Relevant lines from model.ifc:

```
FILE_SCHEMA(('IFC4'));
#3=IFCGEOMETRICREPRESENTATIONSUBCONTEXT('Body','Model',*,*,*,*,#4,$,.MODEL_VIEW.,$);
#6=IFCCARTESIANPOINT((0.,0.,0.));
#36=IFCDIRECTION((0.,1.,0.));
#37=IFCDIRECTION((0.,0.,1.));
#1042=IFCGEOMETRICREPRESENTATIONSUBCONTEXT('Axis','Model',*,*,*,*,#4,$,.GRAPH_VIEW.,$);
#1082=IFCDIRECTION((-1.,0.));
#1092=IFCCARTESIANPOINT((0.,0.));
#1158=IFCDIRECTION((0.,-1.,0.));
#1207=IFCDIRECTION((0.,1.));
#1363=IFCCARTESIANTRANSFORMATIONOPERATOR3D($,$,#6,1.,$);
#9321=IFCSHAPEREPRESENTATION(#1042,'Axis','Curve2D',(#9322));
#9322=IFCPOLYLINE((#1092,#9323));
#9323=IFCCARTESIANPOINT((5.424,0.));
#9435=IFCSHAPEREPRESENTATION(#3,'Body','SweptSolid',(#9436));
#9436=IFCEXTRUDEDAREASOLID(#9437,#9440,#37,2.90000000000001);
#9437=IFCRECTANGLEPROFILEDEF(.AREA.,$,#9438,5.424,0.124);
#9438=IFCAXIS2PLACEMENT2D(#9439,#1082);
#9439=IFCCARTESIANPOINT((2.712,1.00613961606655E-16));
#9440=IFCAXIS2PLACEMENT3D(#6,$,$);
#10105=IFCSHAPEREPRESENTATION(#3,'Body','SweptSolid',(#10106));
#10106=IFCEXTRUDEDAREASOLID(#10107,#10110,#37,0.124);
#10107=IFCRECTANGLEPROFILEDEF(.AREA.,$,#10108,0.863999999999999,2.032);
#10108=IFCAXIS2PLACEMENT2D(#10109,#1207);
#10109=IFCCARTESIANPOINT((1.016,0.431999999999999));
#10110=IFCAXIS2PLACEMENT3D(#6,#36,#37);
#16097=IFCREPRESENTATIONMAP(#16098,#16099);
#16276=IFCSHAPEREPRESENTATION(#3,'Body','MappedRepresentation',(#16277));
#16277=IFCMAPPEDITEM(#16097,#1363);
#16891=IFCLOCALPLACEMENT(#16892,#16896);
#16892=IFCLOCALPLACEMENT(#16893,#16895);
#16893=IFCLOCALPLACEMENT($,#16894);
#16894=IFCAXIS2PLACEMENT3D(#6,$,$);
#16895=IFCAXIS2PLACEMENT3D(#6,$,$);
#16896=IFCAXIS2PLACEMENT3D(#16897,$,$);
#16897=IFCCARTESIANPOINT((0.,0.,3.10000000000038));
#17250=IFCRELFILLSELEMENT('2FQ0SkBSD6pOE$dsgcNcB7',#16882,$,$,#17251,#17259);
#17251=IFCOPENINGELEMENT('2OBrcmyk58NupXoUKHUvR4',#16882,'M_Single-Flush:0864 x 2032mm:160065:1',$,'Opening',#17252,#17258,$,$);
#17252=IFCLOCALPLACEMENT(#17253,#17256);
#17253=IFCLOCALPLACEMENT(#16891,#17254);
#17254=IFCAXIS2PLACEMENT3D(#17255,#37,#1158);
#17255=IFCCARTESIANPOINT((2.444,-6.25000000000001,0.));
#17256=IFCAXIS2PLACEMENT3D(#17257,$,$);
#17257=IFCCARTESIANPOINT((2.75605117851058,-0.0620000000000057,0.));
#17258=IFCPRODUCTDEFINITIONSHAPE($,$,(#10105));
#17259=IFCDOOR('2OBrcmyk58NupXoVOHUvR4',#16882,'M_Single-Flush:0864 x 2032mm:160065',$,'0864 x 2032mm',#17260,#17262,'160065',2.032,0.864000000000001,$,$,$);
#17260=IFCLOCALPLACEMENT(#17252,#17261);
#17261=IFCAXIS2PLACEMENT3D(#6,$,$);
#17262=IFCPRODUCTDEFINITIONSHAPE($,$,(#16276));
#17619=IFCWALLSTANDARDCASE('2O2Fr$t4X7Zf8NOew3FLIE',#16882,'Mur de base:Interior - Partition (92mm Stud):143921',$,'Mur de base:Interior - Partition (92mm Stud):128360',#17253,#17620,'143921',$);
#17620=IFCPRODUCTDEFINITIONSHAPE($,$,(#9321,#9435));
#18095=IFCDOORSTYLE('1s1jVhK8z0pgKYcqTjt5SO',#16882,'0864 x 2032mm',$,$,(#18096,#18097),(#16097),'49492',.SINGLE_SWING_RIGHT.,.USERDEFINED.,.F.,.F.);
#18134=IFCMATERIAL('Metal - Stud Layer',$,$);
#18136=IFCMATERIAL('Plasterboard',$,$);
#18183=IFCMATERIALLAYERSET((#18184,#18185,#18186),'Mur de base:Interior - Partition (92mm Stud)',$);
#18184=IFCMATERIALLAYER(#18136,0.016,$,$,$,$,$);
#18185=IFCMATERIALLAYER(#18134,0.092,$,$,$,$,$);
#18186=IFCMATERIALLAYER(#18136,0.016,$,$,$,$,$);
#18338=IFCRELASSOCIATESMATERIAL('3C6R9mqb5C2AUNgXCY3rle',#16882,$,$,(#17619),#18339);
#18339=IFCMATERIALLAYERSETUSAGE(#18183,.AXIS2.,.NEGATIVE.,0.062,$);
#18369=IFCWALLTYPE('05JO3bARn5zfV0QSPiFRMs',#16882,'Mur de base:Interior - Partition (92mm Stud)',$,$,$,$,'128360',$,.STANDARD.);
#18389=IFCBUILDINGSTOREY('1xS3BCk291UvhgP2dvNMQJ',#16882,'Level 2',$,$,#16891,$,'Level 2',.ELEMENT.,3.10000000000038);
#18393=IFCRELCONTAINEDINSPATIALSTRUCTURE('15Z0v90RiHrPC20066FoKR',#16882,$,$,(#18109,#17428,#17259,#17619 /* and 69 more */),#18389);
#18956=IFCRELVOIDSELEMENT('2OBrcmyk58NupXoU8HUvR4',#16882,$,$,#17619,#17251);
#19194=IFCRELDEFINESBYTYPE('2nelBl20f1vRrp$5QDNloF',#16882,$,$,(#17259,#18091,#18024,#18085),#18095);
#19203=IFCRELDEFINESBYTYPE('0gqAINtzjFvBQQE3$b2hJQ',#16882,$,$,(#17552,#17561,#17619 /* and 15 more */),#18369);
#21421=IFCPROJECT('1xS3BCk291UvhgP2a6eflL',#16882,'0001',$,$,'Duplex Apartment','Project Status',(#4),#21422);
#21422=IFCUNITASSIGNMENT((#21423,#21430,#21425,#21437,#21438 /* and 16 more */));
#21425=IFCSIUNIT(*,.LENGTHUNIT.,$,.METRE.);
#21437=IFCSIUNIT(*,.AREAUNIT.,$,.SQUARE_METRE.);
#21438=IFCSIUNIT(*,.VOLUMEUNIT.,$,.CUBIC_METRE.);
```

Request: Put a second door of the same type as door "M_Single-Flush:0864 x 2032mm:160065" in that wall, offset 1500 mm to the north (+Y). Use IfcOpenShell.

```python
import ifcopenshell
import ifcopenshell.api.feature
import ifcopenshell.api.geometry
import ifcopenshell.api.root
import ifcopenshell.geom
import ifcopenshell.util.element
import ifcopenshell.util.placement
import ifcopenshell.util.shape

model = ifcopenshell.open("model.ifc")
settings = ifcopenshell.geom.settings()


def volume(element):
    """Net volume in cubic metres, openings subtracted."""
    shape = ifcopenshell.geom.create_shape(settings, element)
    return ifcopenshell.util.shape.get_volume(shape.geometry)


def reuse_history(source, copy):
    """copy_class also copies each property set's owner history, people and application; keep the originals."""
    for rel in copy.IsDefinedBy:
        if rel.is_a("IfcRelDefinesByProperties") and (history := rel.RelatingPropertyDefinition.OwnerHistory):
            rel.RelatingPropertyDefinition.OwnerHistory = source.OwnerHistory
            ifcopenshell.util.element.remove_deep2(model, history)


door = model.by_id(17259)
opening = door.FillsVoids[0].RelatingOpeningElement
wall = opening.VoidsElements[0].RelatingBuildingElement
before = volume(wall)
shift = ifcopenshell.util.placement.get_local_placement(wall.ObjectPlacement)[:3, 0] * -1.5

# copy_class copies the void relationship, type, container and properties, but no geometry.
new_opening = ifcopenshell.api.root.copy_class(model, product=opening)
new_opening.Representation = ifcopenshell.util.element.copy_deep(
    model, opening.Representation, exclude=["IfcGeometricRepresentationContext", "IfcRepresentationMap"]
)
new_opening.Name = "M_Single-Flush:0864 x 2032mm"
new_door = ifcopenshell.api.root.copy_class(model, product=door)
new_door.Representation = ifcopenshell.util.element.copy_deep(
    model, door.Representation, exclude=["IfcGeometricRepresentationContext", "IfcRepresentationMap"]
)
new_door.Name = "M_Single-Flush:0864 x 2032mm"
new_door.Tag = None
reuse_history(door, new_door)
ifcopenshell.api.feature.add_filling(model, opening=new_opening, element=new_door)

for old, new in ((opening, new_opening), (door, new_door)):
    matrix = ifcopenshell.util.placement.get_local_placement(old.ObjectPlacement)
    matrix[:3, 3] += shift
    ifcopenshell.api.geometry.edit_object_placement(model, product=new, matrix=matrix, is_si=False)

after = volume(wall)

print(f"wall volume {before:.3f} -> {after:.3f} m3")

model.write("model_edited.ifc")
```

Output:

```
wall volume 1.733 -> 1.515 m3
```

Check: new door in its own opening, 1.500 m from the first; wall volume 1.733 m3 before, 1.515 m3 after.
